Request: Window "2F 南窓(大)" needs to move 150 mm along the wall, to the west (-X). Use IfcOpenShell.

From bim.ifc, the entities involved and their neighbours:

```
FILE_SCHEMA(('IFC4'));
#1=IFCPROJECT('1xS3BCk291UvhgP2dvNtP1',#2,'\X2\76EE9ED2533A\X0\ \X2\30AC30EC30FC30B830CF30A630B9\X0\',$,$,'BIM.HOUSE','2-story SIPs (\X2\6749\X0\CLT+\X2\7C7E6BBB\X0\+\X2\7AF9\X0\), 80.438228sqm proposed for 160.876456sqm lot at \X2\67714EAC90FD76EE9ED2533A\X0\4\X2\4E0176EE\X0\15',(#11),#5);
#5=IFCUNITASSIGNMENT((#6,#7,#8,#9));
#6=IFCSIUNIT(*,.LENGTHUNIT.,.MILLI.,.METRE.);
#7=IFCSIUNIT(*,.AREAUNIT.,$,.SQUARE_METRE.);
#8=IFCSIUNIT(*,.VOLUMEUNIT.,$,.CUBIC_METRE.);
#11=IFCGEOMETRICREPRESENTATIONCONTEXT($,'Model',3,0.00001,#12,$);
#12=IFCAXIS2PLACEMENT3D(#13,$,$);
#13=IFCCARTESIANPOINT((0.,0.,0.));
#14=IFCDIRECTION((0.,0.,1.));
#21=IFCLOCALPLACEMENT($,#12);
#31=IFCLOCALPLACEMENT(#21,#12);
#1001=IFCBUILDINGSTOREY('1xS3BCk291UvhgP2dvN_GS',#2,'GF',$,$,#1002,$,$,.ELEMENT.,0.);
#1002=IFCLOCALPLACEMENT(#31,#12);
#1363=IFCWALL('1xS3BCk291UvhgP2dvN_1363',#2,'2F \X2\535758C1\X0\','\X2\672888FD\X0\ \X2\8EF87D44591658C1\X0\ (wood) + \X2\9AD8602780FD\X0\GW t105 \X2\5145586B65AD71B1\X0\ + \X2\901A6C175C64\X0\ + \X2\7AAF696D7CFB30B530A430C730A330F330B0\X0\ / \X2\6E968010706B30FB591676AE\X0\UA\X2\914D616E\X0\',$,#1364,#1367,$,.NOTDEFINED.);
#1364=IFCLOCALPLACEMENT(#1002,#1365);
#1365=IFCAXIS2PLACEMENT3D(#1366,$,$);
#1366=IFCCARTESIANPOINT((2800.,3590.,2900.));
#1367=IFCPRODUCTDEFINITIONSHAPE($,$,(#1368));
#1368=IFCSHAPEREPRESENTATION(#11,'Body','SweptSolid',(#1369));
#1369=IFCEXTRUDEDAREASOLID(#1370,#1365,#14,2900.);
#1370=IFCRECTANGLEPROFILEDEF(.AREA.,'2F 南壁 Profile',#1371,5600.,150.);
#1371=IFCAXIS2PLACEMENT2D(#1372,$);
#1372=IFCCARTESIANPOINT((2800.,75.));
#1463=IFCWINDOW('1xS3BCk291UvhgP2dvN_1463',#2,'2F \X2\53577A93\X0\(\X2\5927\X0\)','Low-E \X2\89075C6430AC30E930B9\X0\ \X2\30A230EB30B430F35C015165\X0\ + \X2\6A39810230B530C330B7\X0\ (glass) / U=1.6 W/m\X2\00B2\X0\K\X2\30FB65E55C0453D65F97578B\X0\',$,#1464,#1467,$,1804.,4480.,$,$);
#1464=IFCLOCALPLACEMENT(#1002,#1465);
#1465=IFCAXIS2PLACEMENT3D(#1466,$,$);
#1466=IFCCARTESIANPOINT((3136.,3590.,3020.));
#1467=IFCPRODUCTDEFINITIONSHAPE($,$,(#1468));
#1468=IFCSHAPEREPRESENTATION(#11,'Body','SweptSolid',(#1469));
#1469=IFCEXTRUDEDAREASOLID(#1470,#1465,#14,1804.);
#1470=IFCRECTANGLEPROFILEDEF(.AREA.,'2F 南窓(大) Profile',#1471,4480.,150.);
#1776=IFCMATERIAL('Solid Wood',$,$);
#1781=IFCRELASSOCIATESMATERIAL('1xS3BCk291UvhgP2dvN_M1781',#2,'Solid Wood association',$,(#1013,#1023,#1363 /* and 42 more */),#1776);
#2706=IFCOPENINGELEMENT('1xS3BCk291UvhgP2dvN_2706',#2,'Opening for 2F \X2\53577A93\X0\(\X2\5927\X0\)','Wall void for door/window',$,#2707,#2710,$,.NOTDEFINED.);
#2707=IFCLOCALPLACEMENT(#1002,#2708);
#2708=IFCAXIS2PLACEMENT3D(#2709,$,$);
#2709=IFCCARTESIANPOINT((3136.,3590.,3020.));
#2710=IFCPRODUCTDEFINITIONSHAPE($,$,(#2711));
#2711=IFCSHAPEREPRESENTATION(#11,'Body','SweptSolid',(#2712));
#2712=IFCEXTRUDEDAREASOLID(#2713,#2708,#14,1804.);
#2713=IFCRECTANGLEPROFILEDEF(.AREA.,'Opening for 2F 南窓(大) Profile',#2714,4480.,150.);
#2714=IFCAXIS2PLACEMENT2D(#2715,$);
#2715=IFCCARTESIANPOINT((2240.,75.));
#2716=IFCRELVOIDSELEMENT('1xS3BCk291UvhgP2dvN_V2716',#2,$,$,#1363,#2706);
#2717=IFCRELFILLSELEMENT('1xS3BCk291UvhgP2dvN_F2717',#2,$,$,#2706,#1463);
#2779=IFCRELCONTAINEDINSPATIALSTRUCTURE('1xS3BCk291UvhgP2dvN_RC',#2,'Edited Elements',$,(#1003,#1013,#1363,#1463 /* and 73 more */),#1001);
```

```python
import ifcopenshell
import ifcopenshell.api.geometry
import ifcopenshell.util.placement
import ifcopenshell.util.unit

model = ifcopenshell.open("bim.ifc")
unit_scale = ifcopenshell.util.unit.calculate_unit_scale(model)

window = model.by_id(1463)
opening = window.FillsVoids[0].RelatingOpeningElement
wall = opening.VoidsElements[0].RelatingBuildingElement

wall_matrix = ifcopenshell.util.placement.get_local_placement(wall.ObjectPlacement)
shift = wall_matrix[:3, 0] * -0.15 / unit_scale
before = ifcopenshell.util.placement.get_local_placement(window.ObjectPlacement)[:3, 3].copy()

# The window is not placed relative to its opening, so move both.
for product in (opening, window):
    matrix = ifcopenshell.util.placement.get_local_placement(product.ObjectPlacement)
    matrix[:3, 3] += shift
    ifcopenshell.api.geometry.edit_object_placement(model, product=product, matrix=matrix, is_si=False)

after = ifcopenshell.util.placement.get_local_placement(window.ObjectPlacement)[:3, 3]
print("window moved by", (after - before).round(3) + 0.0)

model.write("bim_v2.ifc")
```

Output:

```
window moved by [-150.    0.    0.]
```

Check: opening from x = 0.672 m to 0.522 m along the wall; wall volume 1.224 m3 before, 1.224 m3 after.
